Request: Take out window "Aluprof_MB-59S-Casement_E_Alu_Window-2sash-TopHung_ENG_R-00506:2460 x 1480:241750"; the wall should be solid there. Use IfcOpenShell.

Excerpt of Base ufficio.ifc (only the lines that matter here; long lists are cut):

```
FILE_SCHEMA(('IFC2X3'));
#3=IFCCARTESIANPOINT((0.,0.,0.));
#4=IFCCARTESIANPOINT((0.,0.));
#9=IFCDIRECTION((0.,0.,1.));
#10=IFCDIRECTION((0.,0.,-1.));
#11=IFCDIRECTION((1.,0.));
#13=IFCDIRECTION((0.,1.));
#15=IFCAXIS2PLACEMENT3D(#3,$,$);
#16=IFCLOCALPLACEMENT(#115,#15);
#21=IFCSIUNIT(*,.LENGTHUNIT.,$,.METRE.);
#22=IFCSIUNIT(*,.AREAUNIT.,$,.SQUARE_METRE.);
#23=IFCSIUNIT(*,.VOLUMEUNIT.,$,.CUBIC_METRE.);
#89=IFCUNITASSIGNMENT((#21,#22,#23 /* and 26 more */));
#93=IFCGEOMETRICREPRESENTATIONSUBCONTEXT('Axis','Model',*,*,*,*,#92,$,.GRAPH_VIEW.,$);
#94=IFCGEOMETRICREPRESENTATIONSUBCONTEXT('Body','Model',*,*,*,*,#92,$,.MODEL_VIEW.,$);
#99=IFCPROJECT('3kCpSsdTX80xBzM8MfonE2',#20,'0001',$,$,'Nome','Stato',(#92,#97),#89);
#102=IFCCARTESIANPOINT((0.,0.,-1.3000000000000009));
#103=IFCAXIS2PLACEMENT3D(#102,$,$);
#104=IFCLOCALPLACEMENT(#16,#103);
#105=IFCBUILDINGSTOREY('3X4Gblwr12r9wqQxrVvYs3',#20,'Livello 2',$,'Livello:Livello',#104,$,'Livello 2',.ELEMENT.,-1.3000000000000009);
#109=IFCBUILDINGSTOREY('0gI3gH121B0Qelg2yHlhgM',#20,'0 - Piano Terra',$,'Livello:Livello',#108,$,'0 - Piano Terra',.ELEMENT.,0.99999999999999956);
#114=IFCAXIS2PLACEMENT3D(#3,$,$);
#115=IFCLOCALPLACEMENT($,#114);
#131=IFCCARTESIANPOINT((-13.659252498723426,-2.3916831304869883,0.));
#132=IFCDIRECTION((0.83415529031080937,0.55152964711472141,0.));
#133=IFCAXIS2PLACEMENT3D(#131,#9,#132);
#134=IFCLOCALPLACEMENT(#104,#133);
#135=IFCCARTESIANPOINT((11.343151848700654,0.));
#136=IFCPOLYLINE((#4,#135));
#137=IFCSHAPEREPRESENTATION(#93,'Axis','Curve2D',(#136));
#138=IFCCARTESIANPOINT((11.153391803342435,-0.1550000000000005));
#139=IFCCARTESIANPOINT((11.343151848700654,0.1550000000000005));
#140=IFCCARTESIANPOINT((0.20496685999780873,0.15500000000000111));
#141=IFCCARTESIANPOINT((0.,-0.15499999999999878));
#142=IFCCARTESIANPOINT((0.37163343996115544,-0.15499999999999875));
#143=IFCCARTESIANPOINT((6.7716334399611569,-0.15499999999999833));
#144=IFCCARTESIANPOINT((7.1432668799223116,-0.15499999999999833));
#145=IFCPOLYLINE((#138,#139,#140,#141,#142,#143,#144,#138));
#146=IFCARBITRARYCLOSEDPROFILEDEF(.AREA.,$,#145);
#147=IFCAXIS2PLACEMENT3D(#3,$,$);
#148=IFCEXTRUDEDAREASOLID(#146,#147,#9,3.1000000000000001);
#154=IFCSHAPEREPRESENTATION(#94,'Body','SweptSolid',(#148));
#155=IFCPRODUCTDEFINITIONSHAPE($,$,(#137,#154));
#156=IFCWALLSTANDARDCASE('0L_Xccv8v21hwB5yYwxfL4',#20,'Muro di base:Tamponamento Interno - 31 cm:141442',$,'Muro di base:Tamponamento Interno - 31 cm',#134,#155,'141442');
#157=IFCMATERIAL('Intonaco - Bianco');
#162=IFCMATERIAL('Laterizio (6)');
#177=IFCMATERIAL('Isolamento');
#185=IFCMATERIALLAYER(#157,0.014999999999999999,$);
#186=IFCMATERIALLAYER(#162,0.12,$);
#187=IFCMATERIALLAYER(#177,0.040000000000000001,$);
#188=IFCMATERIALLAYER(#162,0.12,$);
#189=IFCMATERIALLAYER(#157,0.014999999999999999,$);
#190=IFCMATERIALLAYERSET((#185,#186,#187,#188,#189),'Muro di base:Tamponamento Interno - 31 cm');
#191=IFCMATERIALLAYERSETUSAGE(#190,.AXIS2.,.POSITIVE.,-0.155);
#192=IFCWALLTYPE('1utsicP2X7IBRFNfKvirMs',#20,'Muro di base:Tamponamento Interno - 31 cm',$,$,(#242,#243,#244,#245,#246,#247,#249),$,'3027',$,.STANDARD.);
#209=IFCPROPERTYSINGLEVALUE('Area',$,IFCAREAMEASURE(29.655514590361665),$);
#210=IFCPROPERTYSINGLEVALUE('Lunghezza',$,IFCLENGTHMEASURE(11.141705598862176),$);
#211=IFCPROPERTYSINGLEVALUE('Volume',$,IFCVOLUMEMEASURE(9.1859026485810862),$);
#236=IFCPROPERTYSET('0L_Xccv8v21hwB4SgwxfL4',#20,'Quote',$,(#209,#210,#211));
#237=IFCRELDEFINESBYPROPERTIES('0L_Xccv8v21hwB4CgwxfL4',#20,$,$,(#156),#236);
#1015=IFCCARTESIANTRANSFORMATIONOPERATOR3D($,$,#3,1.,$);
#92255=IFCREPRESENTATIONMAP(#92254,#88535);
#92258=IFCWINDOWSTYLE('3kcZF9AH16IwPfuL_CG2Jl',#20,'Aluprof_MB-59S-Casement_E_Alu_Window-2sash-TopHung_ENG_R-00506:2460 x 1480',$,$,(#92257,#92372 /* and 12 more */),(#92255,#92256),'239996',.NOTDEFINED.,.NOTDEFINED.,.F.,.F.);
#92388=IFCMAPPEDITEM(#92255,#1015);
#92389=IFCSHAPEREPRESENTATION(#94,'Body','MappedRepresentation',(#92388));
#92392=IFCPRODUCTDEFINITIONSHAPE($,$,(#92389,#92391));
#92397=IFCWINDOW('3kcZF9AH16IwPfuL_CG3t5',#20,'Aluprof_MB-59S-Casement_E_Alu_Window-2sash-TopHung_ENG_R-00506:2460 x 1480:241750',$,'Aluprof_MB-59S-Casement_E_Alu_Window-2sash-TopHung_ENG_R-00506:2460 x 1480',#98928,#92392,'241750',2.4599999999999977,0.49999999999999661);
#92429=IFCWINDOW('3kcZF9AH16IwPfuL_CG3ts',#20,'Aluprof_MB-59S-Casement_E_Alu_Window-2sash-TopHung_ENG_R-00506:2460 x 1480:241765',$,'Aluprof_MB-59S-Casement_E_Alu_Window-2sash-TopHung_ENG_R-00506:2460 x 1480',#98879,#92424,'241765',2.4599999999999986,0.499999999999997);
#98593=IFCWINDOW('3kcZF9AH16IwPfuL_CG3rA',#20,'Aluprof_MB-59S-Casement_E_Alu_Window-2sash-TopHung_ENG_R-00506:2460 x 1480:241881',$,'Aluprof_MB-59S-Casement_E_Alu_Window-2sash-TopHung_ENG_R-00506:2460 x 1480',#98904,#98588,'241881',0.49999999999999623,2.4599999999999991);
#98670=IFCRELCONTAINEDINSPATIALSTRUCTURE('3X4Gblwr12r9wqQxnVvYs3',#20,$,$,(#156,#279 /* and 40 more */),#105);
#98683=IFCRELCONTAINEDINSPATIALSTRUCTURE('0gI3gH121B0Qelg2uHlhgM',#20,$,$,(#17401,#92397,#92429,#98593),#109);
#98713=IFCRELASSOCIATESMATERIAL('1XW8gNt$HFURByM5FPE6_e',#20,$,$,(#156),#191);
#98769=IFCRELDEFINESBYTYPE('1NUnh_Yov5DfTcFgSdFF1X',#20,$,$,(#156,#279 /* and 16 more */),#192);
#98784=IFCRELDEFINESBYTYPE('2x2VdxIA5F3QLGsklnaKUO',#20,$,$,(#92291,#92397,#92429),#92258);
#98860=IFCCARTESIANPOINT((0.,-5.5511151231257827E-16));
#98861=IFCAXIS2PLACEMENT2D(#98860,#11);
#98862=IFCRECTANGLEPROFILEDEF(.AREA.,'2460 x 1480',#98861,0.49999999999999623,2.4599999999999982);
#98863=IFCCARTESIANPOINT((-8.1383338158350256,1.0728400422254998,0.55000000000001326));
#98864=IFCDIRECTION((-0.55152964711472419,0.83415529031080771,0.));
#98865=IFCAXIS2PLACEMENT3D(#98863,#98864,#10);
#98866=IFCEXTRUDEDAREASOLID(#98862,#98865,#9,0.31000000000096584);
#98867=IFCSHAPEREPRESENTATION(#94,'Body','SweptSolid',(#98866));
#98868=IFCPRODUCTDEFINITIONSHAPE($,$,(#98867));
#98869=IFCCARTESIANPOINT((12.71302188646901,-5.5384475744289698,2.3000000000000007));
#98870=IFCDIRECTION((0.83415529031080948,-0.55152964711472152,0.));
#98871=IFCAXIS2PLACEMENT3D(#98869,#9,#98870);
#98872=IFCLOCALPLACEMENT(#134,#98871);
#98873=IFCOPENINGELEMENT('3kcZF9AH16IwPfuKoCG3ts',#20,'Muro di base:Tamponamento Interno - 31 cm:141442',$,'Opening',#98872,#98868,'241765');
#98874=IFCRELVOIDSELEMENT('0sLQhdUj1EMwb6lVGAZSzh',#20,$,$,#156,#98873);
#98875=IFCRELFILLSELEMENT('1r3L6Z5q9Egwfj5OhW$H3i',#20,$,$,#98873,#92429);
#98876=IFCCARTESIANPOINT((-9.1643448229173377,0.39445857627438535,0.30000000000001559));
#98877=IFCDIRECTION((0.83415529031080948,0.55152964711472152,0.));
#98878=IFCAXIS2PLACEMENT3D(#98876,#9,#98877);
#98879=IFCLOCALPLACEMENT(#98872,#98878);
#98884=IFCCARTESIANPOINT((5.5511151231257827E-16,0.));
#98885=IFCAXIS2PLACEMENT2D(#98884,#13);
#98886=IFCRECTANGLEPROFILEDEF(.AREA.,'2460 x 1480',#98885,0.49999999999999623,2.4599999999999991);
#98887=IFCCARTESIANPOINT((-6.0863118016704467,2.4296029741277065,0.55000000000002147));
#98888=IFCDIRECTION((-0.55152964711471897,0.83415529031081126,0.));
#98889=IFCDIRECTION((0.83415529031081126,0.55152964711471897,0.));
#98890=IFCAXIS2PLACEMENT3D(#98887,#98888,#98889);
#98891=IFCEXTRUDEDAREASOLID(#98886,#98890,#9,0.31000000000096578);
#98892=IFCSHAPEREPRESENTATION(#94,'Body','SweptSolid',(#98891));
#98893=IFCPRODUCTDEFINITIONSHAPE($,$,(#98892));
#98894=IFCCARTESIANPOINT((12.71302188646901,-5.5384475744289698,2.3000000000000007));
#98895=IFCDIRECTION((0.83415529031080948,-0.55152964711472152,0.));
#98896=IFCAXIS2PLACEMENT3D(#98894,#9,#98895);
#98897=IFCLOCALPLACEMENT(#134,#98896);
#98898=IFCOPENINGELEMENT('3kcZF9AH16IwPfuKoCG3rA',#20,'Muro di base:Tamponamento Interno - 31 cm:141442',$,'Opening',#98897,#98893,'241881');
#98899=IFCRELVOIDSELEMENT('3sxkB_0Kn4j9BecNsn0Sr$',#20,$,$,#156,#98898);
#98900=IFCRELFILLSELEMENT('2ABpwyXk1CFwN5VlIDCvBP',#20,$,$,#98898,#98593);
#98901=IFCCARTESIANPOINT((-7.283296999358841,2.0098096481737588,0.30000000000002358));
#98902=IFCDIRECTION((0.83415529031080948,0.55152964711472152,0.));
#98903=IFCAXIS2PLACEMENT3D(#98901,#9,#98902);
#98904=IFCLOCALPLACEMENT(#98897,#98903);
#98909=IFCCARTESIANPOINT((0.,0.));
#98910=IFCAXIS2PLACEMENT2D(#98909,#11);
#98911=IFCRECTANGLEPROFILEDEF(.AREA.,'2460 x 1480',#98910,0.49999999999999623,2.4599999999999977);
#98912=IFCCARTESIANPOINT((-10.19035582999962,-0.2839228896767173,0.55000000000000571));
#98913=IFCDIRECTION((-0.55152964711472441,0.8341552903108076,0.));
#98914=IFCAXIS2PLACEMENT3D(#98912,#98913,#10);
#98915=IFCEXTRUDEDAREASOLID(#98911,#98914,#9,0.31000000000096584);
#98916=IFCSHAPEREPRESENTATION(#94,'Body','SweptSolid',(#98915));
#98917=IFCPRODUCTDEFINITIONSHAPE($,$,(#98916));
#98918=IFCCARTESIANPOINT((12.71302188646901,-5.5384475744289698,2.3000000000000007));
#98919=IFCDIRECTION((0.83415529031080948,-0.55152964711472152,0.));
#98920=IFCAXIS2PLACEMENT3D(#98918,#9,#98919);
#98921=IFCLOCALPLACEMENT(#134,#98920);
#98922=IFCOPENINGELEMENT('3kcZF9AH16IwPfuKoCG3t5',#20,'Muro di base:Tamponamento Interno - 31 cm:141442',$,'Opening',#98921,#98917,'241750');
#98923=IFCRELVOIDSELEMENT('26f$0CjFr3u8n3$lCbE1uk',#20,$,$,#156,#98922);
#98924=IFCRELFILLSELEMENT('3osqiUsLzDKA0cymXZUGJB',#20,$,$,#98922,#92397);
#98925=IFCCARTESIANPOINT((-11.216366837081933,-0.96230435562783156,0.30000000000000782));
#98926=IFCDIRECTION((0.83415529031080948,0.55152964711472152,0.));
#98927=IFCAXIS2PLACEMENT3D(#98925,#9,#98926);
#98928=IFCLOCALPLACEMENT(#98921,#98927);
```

```python
import ifcopenshell
import ifcopenshell.api.feature
import ifcopenshell.api.pset
import ifcopenshell.api.root
import ifcopenshell.geom
import ifcopenshell.util.element
import ifcopenshell.util.shape
import ifcopenshell.util.unit

model = ifcopenshell.open("Base ufficio.ifc")
area_scale = ifcopenshell.util.unit.calculate_unit_scale(model, "AREAUNIT")
volume_scale = ifcopenshell.util.unit.calculate_unit_scale(model, "VOLUMEUNIT")
settings = ifcopenshell.geom.settings()


def volume(element):
    """Net volume in cubic metres, openings subtracted."""
    shape = ifcopenshell.geom.create_shape(settings, element)
    return ifcopenshell.util.shape.get_volume(shape.geometry)


window = model.by_guid("3kcZF9AH16IwPfuL_CG3t5")
opening = window.FillsVoids[0].RelatingOpeningElement
wall = opening.VoidsElements[0].RelatingBuildingElement
before = volume(wall)

ifcopenshell.api.root.remove_product(model, product=window)
ifcopenshell.api.feature.remove_feature(model, feature=opening)

after = volume(wall)
thickness = 0.31  # wall thickness in metres

# Update the wall's stored quantities.
pset = model.by_id(ifcopenshell.util.element.get_pset(wall, "Quote", should_inherit=False)["id"])
ifcopenshell.api.pset.edit_pset(model, pset=pset, properties={
    "Area": model.create_entity("IfcAreaMeasure", after / thickness / area_scale),
    "Volume": model.create_entity("IfcVolumeMeasure", after / volume_scale),
})

print(f"wall volume {before:.3f} -> {after:.3f} m3")

model.write("Base ufficio_edited.ifc")
```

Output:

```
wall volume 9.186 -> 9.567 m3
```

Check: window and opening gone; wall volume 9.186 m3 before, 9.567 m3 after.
